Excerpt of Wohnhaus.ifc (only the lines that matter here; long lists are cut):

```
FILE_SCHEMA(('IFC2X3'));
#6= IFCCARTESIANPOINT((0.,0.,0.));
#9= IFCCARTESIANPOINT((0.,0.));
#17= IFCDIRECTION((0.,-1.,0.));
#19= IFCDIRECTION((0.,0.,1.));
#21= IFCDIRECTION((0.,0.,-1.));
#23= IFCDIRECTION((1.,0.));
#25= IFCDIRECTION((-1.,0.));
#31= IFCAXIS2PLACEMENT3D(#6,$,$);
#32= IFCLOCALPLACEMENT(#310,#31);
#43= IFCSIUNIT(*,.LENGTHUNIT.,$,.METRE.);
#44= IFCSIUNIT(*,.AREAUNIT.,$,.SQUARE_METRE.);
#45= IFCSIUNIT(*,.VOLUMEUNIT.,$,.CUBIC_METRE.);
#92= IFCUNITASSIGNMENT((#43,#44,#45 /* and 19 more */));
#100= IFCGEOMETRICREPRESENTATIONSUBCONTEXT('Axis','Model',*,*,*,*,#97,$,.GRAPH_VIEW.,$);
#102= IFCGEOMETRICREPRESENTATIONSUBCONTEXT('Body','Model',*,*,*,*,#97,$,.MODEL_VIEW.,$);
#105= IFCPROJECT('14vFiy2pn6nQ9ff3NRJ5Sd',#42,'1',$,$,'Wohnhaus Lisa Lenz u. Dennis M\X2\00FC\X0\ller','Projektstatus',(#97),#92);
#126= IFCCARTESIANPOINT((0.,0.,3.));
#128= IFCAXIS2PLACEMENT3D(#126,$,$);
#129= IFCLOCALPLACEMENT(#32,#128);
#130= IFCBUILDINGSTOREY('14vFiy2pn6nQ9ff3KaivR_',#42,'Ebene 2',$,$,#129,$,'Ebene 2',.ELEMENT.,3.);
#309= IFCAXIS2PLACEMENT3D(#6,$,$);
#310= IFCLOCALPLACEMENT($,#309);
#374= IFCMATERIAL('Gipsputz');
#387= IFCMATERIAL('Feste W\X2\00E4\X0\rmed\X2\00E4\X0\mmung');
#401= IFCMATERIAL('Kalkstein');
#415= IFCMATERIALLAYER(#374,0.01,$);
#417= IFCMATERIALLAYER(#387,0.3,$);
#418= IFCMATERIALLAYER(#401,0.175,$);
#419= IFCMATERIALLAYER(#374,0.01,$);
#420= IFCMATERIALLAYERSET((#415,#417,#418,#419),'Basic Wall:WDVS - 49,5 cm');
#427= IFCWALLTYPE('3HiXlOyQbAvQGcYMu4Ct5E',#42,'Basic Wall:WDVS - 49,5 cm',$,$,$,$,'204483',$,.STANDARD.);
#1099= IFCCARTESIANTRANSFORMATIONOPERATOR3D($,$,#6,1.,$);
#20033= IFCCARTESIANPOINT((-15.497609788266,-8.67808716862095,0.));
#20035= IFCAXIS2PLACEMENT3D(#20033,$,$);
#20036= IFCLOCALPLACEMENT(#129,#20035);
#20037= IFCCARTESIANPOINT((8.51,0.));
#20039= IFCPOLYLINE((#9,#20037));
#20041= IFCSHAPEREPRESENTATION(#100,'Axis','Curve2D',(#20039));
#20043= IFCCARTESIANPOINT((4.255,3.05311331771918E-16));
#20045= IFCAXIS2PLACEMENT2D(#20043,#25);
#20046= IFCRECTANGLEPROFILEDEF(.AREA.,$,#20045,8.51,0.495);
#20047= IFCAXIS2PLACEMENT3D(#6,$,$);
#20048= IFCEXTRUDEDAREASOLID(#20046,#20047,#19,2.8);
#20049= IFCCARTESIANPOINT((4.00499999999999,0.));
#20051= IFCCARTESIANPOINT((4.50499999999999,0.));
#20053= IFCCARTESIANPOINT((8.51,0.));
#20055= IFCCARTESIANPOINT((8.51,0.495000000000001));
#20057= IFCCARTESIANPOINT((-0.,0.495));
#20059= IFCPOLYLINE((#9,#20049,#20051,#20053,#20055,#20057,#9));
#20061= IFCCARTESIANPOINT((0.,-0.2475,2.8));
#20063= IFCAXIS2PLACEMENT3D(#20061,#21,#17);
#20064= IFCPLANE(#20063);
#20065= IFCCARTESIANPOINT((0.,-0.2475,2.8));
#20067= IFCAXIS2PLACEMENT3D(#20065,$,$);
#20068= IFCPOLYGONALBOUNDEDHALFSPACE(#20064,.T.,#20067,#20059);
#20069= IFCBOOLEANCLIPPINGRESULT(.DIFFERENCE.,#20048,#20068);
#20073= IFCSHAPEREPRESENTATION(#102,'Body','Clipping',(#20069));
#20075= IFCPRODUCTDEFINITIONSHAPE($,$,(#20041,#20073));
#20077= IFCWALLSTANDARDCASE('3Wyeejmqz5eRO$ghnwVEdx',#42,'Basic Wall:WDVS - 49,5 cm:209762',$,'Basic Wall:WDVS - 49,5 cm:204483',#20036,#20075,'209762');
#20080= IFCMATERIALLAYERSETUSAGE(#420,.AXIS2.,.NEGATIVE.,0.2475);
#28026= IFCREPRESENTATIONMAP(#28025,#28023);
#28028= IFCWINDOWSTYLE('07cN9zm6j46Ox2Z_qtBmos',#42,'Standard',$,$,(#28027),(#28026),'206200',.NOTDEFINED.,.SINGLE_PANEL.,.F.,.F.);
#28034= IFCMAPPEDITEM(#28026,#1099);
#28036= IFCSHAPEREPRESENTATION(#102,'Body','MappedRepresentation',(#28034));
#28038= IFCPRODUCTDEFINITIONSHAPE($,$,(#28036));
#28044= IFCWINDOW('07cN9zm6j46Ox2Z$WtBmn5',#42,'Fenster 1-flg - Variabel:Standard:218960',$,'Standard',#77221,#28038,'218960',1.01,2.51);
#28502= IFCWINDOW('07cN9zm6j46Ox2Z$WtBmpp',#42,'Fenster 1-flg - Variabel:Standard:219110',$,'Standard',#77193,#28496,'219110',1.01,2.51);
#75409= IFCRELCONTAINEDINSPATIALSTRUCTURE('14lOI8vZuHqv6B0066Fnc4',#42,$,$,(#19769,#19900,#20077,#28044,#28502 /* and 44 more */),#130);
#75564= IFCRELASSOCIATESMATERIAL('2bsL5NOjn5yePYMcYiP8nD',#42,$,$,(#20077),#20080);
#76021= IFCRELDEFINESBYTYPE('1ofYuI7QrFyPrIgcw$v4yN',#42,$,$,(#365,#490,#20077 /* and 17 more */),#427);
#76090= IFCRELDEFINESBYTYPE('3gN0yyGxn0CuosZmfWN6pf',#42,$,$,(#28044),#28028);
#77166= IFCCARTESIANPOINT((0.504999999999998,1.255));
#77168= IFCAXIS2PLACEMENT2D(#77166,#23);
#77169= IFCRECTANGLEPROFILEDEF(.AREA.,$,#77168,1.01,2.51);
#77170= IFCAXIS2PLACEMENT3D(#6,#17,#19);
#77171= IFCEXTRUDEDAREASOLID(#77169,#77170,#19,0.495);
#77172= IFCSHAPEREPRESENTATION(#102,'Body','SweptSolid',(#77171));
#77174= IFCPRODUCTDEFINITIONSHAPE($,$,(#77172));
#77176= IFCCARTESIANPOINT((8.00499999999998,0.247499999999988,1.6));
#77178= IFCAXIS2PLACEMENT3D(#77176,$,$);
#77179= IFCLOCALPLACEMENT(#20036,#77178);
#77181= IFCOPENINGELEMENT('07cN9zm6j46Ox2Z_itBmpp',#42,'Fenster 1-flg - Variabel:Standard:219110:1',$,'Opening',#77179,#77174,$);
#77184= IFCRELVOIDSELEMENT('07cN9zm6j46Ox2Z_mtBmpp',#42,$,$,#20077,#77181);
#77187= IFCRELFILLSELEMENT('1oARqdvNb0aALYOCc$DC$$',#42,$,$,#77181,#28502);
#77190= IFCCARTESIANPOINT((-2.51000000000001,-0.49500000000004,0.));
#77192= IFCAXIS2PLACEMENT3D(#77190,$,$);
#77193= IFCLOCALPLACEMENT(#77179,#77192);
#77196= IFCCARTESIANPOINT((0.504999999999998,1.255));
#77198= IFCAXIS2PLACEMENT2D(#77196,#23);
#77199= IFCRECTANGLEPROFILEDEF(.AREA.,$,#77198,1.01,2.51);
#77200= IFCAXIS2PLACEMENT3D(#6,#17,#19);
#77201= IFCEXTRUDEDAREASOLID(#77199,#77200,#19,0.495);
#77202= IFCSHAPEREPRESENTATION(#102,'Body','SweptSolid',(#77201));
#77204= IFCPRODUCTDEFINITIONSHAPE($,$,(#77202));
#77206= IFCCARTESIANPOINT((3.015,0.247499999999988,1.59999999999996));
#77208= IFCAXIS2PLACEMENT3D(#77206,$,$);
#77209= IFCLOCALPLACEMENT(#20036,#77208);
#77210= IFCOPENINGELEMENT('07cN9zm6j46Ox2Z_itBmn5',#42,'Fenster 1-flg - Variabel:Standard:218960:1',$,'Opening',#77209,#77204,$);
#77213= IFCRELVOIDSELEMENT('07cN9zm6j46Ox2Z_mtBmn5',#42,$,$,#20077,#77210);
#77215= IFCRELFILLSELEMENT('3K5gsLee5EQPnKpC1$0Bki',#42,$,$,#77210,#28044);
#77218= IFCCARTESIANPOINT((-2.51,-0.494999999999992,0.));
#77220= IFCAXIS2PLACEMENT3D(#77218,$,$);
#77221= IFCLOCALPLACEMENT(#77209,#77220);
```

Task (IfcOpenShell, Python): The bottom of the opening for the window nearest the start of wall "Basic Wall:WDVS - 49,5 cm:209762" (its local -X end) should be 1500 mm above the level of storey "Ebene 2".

```python
import numpy as np
import ifcopenshell
import ifcopenshell.api.geometry
import ifcopenshell.geom
import ifcopenshell.util.element
import ifcopenshell.util.placement
import ifcopenshell.util.shape
import ifcopenshell.util.unit

model = ifcopenshell.open("Wohnhaus.ifc")
unit_scale = ifcopenshell.util.unit.calculate_unit_scale(model)

window = model.by_guid("07cN9zm6j46Ox2Z$WtBmn5")
opening = window.FillsVoids[0].RelatingOpeningElement
storey = ifcopenshell.util.element.get_container(window, ifc_class="IfcBuildingStorey")
level = ifcopenshell.util.placement.get_local_placement(storey.ObjectPlacement)[2, 3]

# The opening's origin need not be at the sill, so measure its lowest point.
shape = ifcopenshell.geom.create_shape(ifcopenshell.geom.settings(), opening)
bottom = ifcopenshell.util.shape.get_shape_bottom_elevation(shape, shape.geometry) / unit_scale
dz = level + 1.5 - bottom

shift = np.array([0.0, 0.0, dz])
# The window is placed relative to its opening, so it follows when the opening moves.
matrix = ifcopenshell.util.placement.get_local_placement(opening.ObjectPlacement)
matrix[:3, 3] += shift
ifcopenshell.api.geometry.edit_object_placement(
    model, product=opening, matrix=matrix, is_si=False, should_transform_children=True
)

print(f"moved by {dz * unit_scale:+.3f} m")

model.write("Wohnhaus-out.ifc")
```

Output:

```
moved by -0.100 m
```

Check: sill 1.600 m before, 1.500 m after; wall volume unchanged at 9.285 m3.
